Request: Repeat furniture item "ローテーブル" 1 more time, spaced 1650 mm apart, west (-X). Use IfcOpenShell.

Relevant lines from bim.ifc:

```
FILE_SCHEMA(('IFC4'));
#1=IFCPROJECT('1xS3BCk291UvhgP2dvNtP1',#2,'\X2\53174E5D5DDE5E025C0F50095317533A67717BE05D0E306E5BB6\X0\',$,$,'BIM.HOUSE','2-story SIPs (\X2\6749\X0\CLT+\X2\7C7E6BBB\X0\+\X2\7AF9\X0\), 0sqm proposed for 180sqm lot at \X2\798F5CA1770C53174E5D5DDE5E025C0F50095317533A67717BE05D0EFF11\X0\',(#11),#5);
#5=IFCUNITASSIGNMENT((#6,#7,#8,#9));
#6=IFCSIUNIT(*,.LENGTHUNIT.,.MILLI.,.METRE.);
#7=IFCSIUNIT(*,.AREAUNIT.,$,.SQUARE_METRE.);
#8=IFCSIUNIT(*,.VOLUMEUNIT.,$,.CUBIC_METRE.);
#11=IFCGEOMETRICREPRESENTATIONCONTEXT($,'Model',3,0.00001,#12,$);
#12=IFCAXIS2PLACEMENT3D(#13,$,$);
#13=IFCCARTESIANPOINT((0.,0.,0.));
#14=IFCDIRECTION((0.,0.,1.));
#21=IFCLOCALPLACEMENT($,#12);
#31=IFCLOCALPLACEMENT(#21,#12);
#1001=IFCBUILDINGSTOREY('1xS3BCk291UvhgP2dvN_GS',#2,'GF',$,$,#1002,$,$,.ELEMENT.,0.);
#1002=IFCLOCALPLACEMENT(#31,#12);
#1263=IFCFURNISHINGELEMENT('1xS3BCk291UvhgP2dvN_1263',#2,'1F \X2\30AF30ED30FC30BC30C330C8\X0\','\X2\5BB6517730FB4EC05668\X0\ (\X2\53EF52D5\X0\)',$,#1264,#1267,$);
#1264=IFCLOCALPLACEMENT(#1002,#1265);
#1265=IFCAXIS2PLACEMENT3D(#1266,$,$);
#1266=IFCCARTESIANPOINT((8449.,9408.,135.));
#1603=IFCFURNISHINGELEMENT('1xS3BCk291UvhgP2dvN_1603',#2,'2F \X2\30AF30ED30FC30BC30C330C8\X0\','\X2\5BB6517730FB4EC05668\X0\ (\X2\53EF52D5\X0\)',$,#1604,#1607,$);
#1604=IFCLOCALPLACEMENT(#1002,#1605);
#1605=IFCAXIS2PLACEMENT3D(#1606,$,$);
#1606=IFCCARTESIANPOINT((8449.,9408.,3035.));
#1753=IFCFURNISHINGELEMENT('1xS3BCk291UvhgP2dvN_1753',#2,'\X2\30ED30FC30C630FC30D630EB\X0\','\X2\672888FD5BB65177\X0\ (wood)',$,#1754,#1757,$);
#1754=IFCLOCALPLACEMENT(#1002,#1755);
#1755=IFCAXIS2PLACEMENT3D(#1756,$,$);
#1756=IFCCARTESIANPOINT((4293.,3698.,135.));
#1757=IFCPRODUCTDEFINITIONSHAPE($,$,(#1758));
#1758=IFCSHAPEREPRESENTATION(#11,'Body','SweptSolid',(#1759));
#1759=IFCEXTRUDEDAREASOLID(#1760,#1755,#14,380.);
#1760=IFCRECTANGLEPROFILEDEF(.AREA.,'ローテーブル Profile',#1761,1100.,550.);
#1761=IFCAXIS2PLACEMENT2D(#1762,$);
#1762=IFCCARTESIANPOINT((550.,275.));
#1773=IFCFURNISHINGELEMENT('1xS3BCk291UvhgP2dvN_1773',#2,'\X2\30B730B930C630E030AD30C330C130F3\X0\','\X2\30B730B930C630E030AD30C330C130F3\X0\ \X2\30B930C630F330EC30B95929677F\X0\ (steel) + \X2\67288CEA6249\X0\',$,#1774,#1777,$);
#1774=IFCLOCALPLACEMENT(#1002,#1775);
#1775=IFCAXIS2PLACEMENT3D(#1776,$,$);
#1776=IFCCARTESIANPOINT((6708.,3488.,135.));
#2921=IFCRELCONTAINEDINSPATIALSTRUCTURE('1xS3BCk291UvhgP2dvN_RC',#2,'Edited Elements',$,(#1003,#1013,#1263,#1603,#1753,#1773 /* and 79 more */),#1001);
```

```python
import numpy as np
import ifcopenshell
import ifcopenshell.api.geometry
import ifcopenshell.api.root
import ifcopenshell.util.element
import ifcopenshell.util.placement
import ifcopenshell.util.unit

model = ifcopenshell.open("bim.ifc")
unit_scale = ifcopenshell.util.unit.calculate_unit_scale(model)


def reuse_history(source, copy):
    """copy_class also copies each property set's owner history, people and application; keep the originals."""
    for rel in copy.IsDefinedBy:
        if rel.is_a("IfcRelDefinesByProperties") and (history := rel.RelatingPropertyDefinition.OwnerHistory):
            rel.RelatingPropertyDefinition.OwnerHistory = source.OwnerHistory
            ifcopenshell.util.element.remove_deep2(model, history)


source = model.by_guid("1xS3BCk291UvhgP2dvN_1753")
base = ifcopenshell.util.placement.get_local_placement(source.ObjectPlacement)
step = np.array([-1.0, 0.0, 0.0]) * 1.65 / unit_scale

for i in range(1, 2):
    copy = ifcopenshell.api.root.copy_class(model, product=source)
    copy.Representation = ifcopenshell.util.element.copy_deep(
        model, source.Representation, exclude=["IfcGeometricRepresentationContext", "IfcRepresentationMap"]
    )
    reuse_history(source, copy)
    matrix = base.copy()
    matrix[:3, 3] += i * step
    print("added at", matrix[:3, 3].round(3) + 0.0)
    ifcopenshell.api.geometry.edit_object_placement(model, product=copy, matrix=matrix, is_si=False)

model.write("bim_rev.ifc")
```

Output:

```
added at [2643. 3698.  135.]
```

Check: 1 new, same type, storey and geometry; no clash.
